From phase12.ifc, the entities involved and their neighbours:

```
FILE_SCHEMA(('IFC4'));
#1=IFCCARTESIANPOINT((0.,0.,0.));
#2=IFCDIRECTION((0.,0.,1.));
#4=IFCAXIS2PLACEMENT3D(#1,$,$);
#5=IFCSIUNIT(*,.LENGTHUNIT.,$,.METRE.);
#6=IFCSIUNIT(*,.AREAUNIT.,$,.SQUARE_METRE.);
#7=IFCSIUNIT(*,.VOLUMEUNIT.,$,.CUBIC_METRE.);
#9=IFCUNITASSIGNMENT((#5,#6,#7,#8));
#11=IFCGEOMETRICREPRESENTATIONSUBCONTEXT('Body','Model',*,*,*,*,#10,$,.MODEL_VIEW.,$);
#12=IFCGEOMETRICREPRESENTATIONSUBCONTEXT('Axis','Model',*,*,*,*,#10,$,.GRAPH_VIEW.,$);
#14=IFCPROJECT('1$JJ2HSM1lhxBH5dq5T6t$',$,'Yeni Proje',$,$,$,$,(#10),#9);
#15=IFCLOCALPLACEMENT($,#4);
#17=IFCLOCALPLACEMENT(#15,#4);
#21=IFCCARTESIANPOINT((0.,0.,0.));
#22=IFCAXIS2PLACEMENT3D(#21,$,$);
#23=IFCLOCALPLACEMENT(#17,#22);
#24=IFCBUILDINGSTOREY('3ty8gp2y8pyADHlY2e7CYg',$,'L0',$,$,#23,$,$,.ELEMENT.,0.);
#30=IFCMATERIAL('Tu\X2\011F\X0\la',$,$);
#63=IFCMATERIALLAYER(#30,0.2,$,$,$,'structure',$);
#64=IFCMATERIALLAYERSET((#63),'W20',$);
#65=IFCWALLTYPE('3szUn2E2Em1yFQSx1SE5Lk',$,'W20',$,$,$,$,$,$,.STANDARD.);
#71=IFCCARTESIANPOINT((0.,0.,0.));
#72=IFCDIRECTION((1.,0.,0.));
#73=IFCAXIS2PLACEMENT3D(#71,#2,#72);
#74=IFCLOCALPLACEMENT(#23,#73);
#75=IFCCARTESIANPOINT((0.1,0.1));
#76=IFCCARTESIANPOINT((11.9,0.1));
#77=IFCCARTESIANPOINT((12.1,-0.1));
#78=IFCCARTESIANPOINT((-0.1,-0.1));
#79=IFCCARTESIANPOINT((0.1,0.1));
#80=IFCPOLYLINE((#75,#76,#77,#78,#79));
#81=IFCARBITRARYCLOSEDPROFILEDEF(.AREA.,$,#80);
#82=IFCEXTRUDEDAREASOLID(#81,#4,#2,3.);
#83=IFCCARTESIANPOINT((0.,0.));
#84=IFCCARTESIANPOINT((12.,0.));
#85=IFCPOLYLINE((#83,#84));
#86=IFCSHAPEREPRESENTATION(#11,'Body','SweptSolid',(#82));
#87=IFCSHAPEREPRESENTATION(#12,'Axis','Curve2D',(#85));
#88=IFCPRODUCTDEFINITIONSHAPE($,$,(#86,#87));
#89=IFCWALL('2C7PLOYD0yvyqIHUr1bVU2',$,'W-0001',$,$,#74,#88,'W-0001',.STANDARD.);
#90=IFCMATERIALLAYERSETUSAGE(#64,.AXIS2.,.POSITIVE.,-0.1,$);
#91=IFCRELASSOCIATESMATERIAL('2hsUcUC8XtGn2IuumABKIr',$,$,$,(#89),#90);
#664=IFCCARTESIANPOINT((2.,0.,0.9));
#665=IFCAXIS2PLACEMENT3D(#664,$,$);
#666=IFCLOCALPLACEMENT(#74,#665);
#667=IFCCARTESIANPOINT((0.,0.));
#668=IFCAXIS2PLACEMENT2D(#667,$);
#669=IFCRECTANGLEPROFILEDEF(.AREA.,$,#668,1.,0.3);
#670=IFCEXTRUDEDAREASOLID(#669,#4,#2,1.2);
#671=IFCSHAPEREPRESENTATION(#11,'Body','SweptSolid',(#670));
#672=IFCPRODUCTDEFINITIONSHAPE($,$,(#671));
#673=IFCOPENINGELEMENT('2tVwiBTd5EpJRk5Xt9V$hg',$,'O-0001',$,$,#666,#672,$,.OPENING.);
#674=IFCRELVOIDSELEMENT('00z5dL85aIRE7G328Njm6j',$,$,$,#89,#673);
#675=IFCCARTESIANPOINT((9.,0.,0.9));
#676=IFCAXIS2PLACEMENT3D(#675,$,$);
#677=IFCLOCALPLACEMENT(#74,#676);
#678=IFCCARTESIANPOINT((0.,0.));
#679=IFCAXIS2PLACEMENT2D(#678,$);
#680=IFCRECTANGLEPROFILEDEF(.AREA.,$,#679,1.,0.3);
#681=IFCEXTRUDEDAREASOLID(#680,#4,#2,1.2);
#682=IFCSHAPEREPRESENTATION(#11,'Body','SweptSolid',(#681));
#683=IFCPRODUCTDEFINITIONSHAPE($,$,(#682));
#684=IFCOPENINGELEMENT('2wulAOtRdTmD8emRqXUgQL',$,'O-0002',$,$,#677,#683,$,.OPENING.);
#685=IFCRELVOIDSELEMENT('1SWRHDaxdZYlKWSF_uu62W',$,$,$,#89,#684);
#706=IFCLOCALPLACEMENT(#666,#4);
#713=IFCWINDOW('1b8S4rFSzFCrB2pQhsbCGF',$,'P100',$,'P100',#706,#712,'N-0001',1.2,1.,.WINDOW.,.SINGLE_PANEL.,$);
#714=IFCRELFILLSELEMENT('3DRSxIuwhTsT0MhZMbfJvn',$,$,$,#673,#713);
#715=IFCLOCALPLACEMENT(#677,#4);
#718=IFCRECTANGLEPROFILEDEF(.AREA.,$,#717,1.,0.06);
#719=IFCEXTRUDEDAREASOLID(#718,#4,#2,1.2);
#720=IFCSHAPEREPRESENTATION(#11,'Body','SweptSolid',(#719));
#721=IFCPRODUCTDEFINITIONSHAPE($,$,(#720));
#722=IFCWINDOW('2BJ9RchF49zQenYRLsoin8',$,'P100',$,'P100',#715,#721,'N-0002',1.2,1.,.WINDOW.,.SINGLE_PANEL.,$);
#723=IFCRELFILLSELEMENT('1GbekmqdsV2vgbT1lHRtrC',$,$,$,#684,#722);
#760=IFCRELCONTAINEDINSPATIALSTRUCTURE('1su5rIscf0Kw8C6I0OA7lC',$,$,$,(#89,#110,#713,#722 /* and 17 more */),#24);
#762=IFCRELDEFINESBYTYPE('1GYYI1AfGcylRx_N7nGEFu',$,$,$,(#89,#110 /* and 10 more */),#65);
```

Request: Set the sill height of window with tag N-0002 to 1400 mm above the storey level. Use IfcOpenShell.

```python
import numpy as np
import ifcopenshell
import ifcopenshell.api.geometry
import ifcopenshell.geom
import ifcopenshell.util.element
import ifcopenshell.util.placement
import ifcopenshell.util.shape
import ifcopenshell.util.unit

model = ifcopenshell.open("phase12.ifc")
unit_scale = ifcopenshell.util.unit.calculate_unit_scale(model)

window = model.by_guid("2BJ9RchF49zQenYRLsoin8")
opening = window.FillsVoids[0].RelatingOpeningElement
storey = ifcopenshell.util.element.get_container(window, ifc_class="IfcBuildingStorey")
level = ifcopenshell.util.placement.get_local_placement(storey.ObjectPlacement)[2, 3]

# The opening's origin need not be at the sill, so measure its lowest point.
shape = ifcopenshell.geom.create_shape(ifcopenshell.geom.settings(), opening)
bottom = ifcopenshell.util.shape.get_shape_bottom_elevation(shape, shape.geometry) / unit_scale
dz = level + 1.4 - bottom

shift = np.array([0.0, 0.0, dz])
# The window is placed relative to its opening, so it follows when the opening moves.
matrix = ifcopenshell.util.placement.get_local_placement(opening.ObjectPlacement)
matrix[:3, 3] += shift
ifcopenshell.api.geometry.edit_object_placement(
    model, product=opening, matrix=matrix, is_si=False, should_transform_children=True
)

print(f"moved by {dz * unit_scale:+.3f} m")

model.write("phase12_updated.ifc")
```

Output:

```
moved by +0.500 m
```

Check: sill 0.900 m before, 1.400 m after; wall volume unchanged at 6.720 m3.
